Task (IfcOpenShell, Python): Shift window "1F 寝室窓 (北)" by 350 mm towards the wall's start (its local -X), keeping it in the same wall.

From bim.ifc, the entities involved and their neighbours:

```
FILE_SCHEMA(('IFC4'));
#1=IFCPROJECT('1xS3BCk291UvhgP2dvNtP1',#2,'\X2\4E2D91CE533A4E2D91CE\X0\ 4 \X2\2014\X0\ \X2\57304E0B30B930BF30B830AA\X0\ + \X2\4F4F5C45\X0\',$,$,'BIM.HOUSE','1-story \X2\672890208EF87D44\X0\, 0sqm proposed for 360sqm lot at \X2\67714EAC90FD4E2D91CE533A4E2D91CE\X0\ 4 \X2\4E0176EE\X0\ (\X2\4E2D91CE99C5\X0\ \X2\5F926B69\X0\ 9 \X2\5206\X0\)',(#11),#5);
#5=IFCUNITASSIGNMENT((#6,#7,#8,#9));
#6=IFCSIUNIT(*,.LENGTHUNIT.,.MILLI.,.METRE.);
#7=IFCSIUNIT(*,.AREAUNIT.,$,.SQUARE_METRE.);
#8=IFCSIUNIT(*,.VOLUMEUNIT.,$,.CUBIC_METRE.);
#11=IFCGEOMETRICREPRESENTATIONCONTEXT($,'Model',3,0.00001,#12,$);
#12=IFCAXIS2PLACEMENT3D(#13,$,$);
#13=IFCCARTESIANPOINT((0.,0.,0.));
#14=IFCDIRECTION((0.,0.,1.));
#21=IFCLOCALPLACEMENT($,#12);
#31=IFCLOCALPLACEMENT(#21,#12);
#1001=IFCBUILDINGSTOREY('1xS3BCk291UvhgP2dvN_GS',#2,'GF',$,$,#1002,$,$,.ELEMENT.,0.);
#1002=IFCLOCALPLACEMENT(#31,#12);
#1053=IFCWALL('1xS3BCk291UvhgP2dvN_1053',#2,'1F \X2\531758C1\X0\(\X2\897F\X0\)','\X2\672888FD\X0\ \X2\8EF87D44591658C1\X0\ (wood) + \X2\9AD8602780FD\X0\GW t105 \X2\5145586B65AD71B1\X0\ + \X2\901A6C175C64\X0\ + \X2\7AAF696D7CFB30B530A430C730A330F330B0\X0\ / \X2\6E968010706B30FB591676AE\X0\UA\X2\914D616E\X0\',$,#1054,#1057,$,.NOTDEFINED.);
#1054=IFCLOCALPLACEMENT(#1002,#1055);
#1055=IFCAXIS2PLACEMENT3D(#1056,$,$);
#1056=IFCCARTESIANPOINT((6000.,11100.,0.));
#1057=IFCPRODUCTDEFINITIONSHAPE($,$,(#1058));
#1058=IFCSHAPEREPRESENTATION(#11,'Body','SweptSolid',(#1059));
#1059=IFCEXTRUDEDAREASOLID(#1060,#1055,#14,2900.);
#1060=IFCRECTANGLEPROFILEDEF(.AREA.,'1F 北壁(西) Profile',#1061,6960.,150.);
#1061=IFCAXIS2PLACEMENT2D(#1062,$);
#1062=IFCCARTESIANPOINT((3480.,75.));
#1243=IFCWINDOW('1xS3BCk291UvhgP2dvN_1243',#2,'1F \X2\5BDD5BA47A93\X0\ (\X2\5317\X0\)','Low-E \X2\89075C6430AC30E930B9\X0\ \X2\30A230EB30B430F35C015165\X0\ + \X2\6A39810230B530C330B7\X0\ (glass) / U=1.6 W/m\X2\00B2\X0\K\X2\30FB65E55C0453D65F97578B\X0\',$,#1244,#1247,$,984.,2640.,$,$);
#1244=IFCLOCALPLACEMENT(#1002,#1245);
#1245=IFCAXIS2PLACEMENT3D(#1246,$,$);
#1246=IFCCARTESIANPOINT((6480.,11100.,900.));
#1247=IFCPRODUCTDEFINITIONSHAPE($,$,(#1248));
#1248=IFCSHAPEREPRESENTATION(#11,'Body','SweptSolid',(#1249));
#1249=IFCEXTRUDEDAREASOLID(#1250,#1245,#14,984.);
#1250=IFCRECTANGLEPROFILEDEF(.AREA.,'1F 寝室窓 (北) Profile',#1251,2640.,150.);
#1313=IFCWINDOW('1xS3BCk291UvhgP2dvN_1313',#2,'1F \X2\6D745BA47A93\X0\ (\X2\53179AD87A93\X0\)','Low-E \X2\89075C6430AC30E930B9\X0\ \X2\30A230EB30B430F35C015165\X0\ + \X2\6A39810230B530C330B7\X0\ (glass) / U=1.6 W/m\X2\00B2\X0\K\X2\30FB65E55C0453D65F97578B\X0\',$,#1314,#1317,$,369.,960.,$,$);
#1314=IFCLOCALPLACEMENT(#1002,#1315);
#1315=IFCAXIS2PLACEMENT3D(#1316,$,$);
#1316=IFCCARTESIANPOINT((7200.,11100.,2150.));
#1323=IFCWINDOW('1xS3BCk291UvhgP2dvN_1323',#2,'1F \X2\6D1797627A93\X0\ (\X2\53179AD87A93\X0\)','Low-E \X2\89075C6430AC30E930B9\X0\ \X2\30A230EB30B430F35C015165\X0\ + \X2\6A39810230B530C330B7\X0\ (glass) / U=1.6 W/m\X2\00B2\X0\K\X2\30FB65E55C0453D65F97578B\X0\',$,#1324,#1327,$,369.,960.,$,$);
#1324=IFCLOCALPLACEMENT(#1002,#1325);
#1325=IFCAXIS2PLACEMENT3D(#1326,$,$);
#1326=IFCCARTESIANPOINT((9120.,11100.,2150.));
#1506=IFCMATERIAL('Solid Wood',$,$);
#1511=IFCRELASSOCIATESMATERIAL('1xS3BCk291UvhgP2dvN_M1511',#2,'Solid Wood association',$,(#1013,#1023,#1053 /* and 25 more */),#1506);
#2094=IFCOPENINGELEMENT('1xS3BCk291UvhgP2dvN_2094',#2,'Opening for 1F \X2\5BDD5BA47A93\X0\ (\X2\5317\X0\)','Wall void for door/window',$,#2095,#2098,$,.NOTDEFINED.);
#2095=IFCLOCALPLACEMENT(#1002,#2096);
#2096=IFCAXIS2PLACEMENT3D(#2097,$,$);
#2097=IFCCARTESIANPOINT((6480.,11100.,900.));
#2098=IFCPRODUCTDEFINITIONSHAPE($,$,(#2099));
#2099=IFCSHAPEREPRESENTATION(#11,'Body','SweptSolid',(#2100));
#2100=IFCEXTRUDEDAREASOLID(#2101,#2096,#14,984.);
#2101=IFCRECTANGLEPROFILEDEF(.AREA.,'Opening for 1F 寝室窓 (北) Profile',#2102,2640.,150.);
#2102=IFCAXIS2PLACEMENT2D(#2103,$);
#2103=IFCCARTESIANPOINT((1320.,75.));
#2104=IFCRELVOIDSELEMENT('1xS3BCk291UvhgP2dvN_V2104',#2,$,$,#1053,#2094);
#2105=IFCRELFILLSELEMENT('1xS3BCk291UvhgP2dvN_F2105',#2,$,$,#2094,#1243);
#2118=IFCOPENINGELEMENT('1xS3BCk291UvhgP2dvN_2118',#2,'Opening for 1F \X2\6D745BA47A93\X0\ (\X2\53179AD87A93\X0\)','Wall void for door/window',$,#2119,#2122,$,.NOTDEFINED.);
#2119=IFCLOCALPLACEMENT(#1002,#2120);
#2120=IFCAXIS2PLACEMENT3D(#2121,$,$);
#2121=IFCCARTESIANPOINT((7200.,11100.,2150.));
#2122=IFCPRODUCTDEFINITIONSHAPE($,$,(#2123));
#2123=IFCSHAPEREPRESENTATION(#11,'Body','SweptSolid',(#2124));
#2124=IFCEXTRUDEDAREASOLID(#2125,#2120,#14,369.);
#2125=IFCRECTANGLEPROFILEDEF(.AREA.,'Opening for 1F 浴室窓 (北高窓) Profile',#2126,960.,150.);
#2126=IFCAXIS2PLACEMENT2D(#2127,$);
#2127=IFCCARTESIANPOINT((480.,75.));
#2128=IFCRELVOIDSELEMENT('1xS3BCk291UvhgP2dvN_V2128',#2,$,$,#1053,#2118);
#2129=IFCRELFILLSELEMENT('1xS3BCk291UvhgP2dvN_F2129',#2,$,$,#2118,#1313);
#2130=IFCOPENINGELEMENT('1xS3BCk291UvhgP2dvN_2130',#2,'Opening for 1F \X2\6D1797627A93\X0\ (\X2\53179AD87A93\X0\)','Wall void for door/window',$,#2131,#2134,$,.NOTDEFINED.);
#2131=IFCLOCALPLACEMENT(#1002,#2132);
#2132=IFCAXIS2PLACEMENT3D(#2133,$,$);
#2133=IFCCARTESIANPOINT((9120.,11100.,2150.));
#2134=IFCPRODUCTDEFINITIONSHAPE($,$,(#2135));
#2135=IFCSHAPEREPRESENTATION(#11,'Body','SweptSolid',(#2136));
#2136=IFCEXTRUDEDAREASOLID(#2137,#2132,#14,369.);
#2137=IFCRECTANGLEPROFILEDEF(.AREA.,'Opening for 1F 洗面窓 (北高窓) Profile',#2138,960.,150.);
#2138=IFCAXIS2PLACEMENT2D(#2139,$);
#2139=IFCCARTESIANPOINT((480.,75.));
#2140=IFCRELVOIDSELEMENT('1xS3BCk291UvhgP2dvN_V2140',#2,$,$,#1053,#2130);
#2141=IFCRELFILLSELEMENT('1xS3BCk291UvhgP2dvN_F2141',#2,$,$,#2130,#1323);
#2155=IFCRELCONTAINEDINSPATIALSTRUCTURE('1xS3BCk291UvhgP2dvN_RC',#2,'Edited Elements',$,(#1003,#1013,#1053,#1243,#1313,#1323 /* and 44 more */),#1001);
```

```python
import ifcopenshell
import ifcopenshell.api.geometry
import ifcopenshell.util.placement
import ifcopenshell.util.unit

model = ifcopenshell.open("bim.ifc")
unit_scale = ifcopenshell.util.unit.calculate_unit_scale(model)

window = model.by_guid("1xS3BCk291UvhgP2dvN_1243")
opening = window.FillsVoids[0].RelatingOpeningElement
wall = opening.VoidsElements[0].RelatingBuildingElement

wall_matrix = ifcopenshell.util.placement.get_local_placement(wall.ObjectPlacement)
shift = wall_matrix[:3, 0] * -0.35 / unit_scale
before = ifcopenshell.util.placement.get_local_placement(window.ObjectPlacement)[:3, 3].copy()

# The window is not placed relative to its opening, so move both.
for product in (opening, window):
    matrix = ifcopenshell.util.placement.get_local_placement(product.ObjectPlacement)
    matrix[:3, 3] += shift
    ifcopenshell.api.geometry.edit_object_placement(model, product=product, matrix=matrix, is_si=False)

after = ifcopenshell.util.placement.get_local_placement(window.ObjectPlacement)[:3, 3]
print("window moved by", (after - before).round(3) + 0.0)

model.write("bim_edited.ifc")
```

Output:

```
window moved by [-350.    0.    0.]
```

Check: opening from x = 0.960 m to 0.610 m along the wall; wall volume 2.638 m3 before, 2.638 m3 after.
